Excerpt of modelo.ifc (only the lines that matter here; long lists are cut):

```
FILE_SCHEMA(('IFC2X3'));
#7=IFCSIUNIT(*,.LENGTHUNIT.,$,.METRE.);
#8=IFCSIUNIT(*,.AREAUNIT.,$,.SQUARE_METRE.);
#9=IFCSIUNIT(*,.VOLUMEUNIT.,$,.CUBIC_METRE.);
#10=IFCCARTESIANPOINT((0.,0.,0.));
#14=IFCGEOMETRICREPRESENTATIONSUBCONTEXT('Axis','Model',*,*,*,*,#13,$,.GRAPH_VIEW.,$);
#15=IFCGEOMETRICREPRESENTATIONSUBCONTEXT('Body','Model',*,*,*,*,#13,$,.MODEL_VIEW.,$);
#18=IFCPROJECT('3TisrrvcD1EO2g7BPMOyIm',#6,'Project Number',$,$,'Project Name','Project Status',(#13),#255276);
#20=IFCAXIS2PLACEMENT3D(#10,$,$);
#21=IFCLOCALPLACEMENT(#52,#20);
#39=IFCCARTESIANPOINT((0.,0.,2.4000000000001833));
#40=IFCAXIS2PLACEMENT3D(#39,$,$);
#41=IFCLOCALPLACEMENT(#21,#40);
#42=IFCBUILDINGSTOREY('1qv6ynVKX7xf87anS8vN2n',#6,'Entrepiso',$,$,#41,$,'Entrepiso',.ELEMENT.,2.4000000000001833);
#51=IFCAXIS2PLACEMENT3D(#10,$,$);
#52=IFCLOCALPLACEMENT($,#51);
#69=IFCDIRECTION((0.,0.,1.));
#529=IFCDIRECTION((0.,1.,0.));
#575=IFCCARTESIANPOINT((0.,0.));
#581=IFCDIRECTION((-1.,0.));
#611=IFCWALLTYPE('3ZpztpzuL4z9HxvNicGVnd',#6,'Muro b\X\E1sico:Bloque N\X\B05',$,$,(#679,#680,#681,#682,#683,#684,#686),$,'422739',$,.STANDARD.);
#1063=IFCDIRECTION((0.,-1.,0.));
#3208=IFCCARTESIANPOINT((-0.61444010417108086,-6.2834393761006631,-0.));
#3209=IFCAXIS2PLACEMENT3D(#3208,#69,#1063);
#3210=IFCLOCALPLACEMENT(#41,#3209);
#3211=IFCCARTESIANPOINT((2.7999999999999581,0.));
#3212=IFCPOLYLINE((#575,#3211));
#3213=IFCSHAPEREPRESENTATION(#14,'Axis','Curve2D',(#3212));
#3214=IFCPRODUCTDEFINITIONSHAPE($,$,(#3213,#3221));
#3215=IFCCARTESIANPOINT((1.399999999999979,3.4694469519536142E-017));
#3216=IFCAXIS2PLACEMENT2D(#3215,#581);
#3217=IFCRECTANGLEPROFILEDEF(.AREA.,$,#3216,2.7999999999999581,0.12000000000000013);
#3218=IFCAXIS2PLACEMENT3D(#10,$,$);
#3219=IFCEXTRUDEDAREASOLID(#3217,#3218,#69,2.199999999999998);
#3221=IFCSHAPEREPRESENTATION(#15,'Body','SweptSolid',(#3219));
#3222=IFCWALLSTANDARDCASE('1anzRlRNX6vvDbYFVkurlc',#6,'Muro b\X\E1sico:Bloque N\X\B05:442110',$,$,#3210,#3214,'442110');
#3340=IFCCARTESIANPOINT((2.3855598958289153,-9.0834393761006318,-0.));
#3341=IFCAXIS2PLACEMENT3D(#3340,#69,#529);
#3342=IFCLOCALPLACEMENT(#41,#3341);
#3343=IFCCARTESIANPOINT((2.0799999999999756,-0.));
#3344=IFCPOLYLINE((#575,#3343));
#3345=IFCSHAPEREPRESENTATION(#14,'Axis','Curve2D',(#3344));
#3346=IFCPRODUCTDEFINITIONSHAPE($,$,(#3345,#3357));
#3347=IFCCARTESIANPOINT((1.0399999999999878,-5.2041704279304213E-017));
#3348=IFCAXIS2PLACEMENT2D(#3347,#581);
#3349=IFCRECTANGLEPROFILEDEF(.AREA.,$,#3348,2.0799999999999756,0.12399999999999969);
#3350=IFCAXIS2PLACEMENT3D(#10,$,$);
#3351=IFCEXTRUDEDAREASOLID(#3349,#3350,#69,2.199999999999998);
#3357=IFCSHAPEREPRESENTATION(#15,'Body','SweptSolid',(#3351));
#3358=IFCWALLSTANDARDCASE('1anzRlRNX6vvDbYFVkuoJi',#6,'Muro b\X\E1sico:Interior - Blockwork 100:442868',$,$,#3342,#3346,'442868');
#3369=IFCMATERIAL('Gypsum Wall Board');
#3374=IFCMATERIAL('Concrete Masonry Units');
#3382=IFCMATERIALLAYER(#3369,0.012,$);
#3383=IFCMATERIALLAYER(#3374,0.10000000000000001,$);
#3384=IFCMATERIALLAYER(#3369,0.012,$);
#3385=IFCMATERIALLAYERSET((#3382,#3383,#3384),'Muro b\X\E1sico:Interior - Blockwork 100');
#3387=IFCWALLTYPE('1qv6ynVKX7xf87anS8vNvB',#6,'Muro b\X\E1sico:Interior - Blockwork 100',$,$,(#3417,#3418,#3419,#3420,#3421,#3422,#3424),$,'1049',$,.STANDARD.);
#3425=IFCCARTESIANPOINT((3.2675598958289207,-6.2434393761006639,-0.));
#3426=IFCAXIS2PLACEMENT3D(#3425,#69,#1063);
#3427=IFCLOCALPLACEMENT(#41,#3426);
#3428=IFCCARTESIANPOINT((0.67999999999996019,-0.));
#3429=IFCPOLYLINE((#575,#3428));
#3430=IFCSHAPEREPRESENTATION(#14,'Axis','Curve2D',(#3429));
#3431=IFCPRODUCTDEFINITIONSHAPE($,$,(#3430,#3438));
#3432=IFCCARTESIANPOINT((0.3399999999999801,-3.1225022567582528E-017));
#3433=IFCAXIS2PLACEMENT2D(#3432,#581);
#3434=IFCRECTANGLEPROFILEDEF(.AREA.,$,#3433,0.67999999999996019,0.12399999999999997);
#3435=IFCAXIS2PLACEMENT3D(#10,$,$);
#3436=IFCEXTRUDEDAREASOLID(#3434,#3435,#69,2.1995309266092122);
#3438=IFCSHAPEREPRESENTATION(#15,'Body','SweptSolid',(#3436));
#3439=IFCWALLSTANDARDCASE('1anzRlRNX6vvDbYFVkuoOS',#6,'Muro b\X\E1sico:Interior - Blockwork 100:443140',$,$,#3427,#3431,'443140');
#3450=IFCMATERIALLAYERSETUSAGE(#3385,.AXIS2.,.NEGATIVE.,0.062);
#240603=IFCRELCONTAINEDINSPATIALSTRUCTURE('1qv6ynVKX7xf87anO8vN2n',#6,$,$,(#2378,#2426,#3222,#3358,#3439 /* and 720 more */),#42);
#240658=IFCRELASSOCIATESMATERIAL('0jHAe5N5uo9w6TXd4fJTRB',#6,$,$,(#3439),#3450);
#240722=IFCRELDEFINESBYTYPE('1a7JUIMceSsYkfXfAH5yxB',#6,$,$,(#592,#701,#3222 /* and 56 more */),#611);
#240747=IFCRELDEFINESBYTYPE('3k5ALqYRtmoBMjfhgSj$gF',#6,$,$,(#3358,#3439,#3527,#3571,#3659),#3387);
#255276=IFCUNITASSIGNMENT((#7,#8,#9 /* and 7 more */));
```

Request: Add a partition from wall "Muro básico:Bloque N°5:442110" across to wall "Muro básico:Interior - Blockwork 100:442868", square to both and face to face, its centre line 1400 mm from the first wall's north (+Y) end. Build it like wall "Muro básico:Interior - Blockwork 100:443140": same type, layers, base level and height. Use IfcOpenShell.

```python
import numpy as np
import ifcopenshell
import ifcopenshell.api.geometry
import ifcopenshell.api.material
import ifcopenshell.api.pset
import ifcopenshell.api.root
import ifcopenshell.api.spatial
import ifcopenshell.api.type
import ifcopenshell.geom
import ifcopenshell.util.element
import ifcopenshell.util.placement
import ifcopenshell.util.representation
import ifcopenshell.util.shape
import ifcopenshell.util.unit

model = ifcopenshell.open("modelo.ifc")
unit_scale = ifcopenshell.util.unit.calculate_unit_scale(model)
settings = ifcopenshell.geom.settings()
settings.set("use-world-coords", True)

start_wall = model.by_id(3222)
end_wall = model.by_id(3358)
like = model.by_guid("1anzRlRNX6vvDbYFVkuoOS")
matrix = ifcopenshell.util.placement.get_local_placement(start_wall.ObjectPlacement)
matrix[:3, 3] *= unit_scale


def extent(element):
    """Bounding box in the first wall's axes, in metres."""
    shape = ifcopenshell.geom.create_shape(settings, element)
    points = (ifcopenshell.util.shape.get_vertices(shape.geometry) - matrix[:3, 3]) @ matrix[:3, :3]
    return points.min(axis=0), points.max(axis=0)


y_start = extent(start_wall)[1][1]
y_end = extent(end_wall)[0][1]
like_min, like_max = extent(like)
length, height = float(abs(y_end - y_start)), float(like_max[2] - like_min[2])
layer_set = ifcopenshell.util.element.get_material(like, should_skip_usage=True)
thickness = sum(layer.LayerThickness for layer in layer_set.MaterialLayers) * unit_scale

wall = ifcopenshell.api.root.create_entity(model, ifc_class="IfcWallStandardCase", name="New partition")
storey = ifcopenshell.util.element.get_container(like)
ifcopenshell.api.spatial.assign_container(model, products=[wall], relating_structure=storey)
ifcopenshell.api.type.assign_type(
    model, related_objects=[wall], relating_type=ifcopenshell.util.element.get_type(like), should_map_representations=False
)
rel = ifcopenshell.api.material.assign_material(
    model, products=[wall], type="IfcMaterialLayerSetUsage", material=layer_set
)
rel.RelatingMaterial.OffsetFromReferenceLine = -thickness / 2 / unit_scale
pset = ifcopenshell.api.pset.add_pset(model, product=wall, name="Pset_WallCommon")
ifcopenshell.api.pset.edit_pset(model, pset=pset, properties={"IsExternal": False, "LoadBearing": False})

# The axis runs down the middle of the wall.
axis = ifcopenshell.api.geometry.add_axis_representation(
    model, context=ifcopenshell.util.representation.get_context(model, "Model", "Axis"), axis=[(0.0, 0.0), (length, 0.0)]
)
body = ifcopenshell.api.geometry.add_wall_representation(
    model,
    context=ifcopenshell.util.representation.get_context(model, "Model", "Body", "MODEL_VIEW"),
    length=length,
    height=height,
    thickness=thickness,
    offset=-thickness / 2,
)
for representation in (axis, body):
    ifcopenshell.api.geometry.assign_representation(model, product=wall, representation=representation)

placement = matrix @ ifcopenshell.util.placement.rotation(90, "Z")
placement[:, 3] = matrix @ np.array([extent(start_wall)[0][0] + 1.4, y_start, like_min[2], 1.0])
ifcopenshell.api.geometry.edit_object_placement(model, product=wall, matrix=placement)

print(f"partition {length:.3f} m long, {height:.3f} m high, {thickness:.3f} m thick")

model.write("modelo_rev.ifc")
```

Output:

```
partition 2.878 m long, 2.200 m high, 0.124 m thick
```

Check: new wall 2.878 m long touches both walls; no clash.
